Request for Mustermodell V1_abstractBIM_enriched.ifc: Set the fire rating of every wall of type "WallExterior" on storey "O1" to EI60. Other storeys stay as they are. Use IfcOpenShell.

First a look at what the model holds.

```python
import ifcopenshell
import ifcopenshell.util.element

model = ifcopenshell.open("Mustermodell V1_abstractBIM_enriched.ifc")
print(model.schema)
storey = next(s for s in model.by_type("IfcBuildingStorey") if s.Name == "O1")
walls = [e for e in ifcopenshell.util.element.get_decomposition(storey) if e.is_a("IfcWall")]
seen = {}
for e in walls:
    element_type = ifcopenshell.util.element.get_type(e)
    key = (element_type.Name if element_type != e and element_type else None, ifcopenshell.util.element.get_pset(e, "Pset_WallCommon", "FireRating"))
    seen[key] = seen.get(key, 0) + 1
for (name, value), count in sorted(seen.items(), key=str):
    print(count, "x", name, "|", value)
```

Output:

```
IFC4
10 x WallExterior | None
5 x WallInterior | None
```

```python
import ifcopenshell
import ifcopenshell.api.pset
import ifcopenshell.util.element

model = ifcopenshell.open("Mustermodell V1_abstractBIM_enriched.ifc")

storey = next(s for s in model.by_type("IfcBuildingStorey") if s.Name == "O1")
walls = [e for e in ifcopenshell.util.element.get_decomposition(storey) if e.is_a("IfcWall")]

count = 0
for e in walls:
    element_type = ifcopenshell.util.element.get_type(e)
    if element_type in (None, e) or element_type.Name != "WallExterior":
        continue
    # add_pset returns the element's existing set when there is one.
    pset = ifcopenshell.api.pset.add_pset(model, product=e, name="Pset_WallCommon")
    ifcopenshell.api.pset.edit_pset(model, pset=pset, properties={"FireRating": "EI60"})
    count += 1

print(count, "walls updated")

model.write("Mustermodell V1_abstractBIM_enriched_updated.ifc")
```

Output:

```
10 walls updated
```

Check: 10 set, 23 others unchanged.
